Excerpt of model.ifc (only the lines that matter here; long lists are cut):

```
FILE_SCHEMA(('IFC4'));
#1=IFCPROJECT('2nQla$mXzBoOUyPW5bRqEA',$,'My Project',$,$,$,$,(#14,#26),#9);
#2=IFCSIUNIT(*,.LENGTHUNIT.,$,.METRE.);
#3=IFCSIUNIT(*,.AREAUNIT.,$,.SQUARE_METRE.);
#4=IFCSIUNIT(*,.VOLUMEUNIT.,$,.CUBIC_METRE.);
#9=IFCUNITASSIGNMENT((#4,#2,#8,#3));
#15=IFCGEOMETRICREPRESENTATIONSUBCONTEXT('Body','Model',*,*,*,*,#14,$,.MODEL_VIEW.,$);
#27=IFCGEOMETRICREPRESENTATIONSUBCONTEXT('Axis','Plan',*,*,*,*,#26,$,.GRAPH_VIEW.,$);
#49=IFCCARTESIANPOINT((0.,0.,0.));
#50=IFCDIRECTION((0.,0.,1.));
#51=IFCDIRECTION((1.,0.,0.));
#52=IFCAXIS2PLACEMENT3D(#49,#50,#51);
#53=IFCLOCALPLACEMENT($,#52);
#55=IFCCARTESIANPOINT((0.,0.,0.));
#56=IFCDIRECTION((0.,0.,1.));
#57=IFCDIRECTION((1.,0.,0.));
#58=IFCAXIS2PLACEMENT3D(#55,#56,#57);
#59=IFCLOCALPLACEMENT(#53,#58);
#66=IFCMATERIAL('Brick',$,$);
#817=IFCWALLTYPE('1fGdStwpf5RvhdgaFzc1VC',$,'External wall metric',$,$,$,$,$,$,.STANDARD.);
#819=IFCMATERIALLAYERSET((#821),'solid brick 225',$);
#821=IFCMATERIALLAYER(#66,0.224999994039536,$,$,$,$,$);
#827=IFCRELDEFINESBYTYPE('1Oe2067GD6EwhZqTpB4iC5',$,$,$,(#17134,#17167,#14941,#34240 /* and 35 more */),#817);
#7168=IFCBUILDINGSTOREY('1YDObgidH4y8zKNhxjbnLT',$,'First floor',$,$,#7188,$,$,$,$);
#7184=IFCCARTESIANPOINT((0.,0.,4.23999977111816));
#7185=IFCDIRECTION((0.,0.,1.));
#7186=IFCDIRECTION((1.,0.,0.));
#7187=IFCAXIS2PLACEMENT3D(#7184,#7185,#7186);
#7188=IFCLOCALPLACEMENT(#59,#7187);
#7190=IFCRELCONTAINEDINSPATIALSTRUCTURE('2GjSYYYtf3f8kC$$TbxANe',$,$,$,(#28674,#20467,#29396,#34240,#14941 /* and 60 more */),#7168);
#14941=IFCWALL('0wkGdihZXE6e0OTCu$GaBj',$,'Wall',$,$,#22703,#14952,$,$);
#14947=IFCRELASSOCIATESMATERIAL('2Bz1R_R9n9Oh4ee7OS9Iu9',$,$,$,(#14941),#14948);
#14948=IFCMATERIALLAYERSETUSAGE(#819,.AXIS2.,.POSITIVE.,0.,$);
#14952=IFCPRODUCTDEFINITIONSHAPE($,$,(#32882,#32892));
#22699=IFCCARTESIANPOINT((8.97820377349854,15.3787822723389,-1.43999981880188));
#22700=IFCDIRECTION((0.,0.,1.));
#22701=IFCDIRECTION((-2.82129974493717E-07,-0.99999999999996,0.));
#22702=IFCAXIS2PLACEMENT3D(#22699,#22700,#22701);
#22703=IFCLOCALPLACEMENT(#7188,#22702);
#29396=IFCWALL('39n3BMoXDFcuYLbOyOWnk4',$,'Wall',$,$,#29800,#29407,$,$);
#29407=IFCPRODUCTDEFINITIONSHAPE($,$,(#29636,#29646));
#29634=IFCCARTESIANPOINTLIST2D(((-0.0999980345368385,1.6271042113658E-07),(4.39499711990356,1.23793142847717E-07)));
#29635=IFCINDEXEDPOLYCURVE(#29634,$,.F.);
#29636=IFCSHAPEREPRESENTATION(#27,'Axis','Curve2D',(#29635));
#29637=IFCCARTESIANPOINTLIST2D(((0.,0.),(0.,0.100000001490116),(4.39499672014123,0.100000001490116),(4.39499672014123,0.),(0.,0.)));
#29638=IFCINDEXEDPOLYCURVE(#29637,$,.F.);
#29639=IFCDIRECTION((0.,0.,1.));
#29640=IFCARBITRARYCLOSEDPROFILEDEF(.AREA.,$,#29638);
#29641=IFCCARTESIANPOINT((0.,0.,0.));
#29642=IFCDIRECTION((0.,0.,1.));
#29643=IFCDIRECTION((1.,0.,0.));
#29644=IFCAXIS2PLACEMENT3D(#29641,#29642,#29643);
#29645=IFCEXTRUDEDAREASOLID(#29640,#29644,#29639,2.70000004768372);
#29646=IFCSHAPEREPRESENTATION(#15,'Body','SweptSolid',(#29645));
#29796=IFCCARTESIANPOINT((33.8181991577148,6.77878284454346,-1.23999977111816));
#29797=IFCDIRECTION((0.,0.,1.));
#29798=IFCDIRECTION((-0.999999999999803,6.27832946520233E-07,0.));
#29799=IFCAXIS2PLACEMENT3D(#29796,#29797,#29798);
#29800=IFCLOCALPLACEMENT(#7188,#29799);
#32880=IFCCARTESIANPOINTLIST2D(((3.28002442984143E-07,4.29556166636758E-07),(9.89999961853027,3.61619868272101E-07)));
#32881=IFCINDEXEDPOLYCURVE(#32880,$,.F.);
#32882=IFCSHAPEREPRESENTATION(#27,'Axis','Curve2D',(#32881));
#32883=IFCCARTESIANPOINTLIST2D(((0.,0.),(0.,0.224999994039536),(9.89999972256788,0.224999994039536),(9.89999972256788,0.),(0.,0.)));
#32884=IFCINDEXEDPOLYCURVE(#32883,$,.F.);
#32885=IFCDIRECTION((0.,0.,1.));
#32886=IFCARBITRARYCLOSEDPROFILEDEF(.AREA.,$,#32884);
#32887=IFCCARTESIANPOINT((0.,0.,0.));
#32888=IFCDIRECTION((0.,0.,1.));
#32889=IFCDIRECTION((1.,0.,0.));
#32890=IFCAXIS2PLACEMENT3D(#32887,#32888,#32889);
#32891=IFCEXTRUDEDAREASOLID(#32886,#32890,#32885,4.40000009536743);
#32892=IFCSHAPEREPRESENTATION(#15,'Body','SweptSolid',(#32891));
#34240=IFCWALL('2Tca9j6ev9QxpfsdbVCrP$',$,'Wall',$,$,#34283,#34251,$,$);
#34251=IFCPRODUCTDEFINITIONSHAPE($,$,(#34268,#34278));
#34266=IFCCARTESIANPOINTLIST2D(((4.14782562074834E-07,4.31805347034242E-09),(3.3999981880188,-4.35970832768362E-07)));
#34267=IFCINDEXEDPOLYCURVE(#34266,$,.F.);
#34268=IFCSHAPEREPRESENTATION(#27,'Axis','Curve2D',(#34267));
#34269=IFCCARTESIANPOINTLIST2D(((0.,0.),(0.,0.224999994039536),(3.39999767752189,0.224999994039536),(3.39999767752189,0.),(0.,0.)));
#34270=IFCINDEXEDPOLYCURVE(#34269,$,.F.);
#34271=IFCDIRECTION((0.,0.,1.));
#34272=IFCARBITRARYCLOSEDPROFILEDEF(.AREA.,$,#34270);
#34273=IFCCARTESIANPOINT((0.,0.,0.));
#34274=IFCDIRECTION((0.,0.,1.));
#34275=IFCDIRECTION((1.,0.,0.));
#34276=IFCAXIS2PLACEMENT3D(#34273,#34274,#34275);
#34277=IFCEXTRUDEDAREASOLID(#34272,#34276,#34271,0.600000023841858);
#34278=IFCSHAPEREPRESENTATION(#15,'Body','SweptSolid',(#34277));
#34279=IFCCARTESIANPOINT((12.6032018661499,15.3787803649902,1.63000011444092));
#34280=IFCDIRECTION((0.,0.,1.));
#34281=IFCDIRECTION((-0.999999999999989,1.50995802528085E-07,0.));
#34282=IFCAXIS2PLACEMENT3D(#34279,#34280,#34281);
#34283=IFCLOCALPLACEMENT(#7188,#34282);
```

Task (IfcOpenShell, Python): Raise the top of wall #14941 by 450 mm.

```python
import ifcopenshell
import ifcopenshell.geom
import ifcopenshell.util.representation
import ifcopenshell.util.shape

model = ifcopenshell.open("model.ifc")
settings = ifcopenshell.geom.settings()


def volume(element):
    """Net volume in cubic metres, openings subtracted."""
    shape = ifcopenshell.geom.create_shape(settings, element)
    return ifcopenshell.util.shape.get_volume(shape.geometry)


wall = model.by_id(14941)
before = volume(wall)

body = ifcopenshell.util.representation.get_representation(wall, "Model", "Body")
solid = body.Items[0]
old_height = solid.Depth
solid.Depth += 0.45
after = volume(wall)

print(f"height {old_height:g} -> {solid.Depth:g}, volume {before:.3f} -> {after:.3f} m3")

model.write("model_v2.ifc")
```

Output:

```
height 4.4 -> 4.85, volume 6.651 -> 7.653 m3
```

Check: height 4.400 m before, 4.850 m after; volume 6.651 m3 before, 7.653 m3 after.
